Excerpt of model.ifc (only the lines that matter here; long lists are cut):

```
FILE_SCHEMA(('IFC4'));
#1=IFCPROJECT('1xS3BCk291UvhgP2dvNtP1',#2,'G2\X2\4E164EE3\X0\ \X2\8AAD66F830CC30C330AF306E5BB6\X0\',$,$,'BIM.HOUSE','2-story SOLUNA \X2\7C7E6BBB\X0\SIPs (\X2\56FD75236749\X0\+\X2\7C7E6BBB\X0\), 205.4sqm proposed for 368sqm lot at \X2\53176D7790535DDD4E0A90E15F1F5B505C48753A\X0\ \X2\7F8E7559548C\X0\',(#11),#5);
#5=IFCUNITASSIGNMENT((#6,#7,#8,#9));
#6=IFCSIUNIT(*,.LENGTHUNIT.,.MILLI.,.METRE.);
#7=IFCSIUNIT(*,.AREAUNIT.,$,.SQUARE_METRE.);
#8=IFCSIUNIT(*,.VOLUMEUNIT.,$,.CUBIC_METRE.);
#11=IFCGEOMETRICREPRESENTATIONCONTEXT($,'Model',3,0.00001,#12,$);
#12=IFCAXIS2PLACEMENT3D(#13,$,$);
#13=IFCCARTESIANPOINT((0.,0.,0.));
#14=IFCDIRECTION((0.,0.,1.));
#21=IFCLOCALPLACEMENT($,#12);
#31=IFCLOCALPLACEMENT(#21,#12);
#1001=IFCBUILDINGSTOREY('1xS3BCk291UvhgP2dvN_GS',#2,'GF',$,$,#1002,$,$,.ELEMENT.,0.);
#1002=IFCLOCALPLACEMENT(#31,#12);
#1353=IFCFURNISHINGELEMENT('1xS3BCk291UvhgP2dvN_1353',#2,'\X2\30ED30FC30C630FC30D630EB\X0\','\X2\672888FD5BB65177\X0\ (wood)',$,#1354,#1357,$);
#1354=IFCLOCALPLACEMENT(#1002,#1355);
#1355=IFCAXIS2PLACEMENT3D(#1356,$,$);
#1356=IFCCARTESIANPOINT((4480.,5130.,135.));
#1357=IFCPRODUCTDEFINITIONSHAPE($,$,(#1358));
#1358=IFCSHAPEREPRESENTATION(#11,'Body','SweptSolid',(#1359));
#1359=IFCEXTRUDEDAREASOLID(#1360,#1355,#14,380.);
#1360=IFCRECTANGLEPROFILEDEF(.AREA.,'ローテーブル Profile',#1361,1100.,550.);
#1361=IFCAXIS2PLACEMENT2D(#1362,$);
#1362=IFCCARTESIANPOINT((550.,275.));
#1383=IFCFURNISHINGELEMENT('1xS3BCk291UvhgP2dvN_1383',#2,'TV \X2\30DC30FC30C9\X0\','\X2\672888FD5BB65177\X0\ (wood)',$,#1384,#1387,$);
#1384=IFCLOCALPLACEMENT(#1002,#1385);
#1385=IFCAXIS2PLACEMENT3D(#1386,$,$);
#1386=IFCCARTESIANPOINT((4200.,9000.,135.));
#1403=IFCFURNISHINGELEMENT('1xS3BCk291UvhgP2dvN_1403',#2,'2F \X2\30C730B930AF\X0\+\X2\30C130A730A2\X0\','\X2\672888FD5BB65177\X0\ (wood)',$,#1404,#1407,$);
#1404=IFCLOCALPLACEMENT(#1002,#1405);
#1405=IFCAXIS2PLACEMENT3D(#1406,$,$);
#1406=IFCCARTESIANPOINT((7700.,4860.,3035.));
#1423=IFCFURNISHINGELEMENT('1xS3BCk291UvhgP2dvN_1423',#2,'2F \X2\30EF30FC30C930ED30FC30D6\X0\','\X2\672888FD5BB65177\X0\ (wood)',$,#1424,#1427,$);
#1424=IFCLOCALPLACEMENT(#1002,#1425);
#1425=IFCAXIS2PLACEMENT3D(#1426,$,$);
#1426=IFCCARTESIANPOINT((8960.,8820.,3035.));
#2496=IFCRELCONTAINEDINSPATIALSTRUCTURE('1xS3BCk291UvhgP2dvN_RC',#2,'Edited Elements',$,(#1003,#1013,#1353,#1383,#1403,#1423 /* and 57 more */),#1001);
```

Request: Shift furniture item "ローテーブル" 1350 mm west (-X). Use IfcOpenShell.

```python
import ifcopenshell
import ifcopenshell.api.geometry
import ifcopenshell.util.placement
import ifcopenshell.util.unit

model = ifcopenshell.open("model.ifc")
unit_scale = ifcopenshell.util.unit.calculate_unit_scale(model)

item = model.by_guid("1xS3BCk291UvhgP2dvN_1353")
matrix = ifcopenshell.util.placement.get_local_placement(item.ObjectPlacement)
matrix[0, 3] -= 1.35 / unit_scale
ifcopenshell.api.geometry.edit_object_placement(model, product=item, matrix=matrix, is_si=False)

print(ifcopenshell.util.placement.get_local_placement(item.ObjectPlacement).round(3) + 0.0)

model.write("model_rev.ifc")
```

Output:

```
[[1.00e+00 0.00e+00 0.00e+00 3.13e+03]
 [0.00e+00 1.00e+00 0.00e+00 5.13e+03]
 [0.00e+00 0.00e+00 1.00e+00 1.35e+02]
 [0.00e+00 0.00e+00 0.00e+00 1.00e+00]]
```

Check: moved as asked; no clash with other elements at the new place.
